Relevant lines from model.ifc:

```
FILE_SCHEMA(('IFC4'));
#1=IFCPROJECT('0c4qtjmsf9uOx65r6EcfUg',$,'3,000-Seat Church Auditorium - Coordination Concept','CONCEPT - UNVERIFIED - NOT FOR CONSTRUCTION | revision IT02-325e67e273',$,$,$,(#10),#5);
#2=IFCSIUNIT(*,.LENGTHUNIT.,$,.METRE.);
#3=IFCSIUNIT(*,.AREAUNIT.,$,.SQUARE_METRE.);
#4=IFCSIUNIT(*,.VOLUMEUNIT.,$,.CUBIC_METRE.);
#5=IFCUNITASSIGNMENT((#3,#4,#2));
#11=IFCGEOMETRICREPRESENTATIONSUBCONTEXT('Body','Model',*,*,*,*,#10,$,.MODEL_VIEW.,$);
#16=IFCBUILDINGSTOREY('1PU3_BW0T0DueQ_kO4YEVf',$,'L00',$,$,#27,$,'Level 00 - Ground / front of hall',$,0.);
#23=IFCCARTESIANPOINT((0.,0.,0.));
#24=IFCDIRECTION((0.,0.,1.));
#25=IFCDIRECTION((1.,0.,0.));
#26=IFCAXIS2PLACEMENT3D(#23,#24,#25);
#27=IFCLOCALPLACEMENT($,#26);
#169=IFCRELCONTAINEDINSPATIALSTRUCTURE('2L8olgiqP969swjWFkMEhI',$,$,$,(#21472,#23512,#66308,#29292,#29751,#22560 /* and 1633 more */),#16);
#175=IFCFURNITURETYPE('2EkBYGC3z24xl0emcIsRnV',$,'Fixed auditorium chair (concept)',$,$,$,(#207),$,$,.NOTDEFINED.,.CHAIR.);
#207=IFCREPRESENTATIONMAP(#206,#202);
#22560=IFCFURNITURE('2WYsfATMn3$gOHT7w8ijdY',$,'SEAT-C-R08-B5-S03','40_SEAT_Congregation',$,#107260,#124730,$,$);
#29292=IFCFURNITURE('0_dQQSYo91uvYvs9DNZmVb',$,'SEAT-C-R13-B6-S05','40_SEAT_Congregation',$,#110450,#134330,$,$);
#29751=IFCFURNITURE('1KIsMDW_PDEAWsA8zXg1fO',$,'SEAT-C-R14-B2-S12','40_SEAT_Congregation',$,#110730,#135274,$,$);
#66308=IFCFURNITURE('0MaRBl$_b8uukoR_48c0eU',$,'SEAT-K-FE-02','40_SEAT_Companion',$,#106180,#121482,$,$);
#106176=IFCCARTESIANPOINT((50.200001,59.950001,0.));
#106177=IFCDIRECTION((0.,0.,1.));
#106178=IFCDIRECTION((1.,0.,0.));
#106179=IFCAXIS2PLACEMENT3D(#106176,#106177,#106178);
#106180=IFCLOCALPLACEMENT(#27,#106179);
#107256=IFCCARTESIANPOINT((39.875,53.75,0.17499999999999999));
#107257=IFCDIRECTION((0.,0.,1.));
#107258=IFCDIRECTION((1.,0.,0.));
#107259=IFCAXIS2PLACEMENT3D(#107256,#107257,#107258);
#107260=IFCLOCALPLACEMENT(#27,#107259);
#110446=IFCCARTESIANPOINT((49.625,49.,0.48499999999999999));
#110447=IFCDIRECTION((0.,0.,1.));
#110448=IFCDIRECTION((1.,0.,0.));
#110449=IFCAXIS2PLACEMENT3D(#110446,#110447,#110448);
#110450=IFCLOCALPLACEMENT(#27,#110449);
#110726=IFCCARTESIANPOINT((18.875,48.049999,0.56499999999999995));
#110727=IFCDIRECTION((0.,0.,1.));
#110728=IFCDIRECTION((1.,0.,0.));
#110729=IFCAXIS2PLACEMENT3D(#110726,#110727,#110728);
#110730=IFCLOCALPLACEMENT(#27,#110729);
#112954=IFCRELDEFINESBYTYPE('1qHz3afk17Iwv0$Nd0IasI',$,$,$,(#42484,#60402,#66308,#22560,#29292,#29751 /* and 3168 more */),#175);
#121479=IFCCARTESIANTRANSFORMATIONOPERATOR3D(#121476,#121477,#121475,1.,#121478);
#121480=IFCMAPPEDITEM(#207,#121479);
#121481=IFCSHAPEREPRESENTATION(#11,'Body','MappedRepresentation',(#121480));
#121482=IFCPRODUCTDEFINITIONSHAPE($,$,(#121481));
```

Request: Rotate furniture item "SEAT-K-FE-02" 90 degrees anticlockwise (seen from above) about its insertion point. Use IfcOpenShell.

```python
import ifcopenshell
import ifcopenshell.api.geometry
import ifcopenshell.util.placement

model = ifcopenshell.open("model.ifc")

item = model.by_guid("0MaRBl$_b8uukoR_48c0eU")
matrix = ifcopenshell.util.placement.get_local_placement(item.ObjectPlacement)
matrix = matrix @ ifcopenshell.util.placement.rotation(90, "Z")
ifcopenshell.api.geometry.edit_object_placement(model, product=item, matrix=matrix, is_si=False)

print(ifcopenshell.util.placement.get_local_placement(item.ObjectPlacement).round(3) + 0.0)

model.write("model-out.ifc")
```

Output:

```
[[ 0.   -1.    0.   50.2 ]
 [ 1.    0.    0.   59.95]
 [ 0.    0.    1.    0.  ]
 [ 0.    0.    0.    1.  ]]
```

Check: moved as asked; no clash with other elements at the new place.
